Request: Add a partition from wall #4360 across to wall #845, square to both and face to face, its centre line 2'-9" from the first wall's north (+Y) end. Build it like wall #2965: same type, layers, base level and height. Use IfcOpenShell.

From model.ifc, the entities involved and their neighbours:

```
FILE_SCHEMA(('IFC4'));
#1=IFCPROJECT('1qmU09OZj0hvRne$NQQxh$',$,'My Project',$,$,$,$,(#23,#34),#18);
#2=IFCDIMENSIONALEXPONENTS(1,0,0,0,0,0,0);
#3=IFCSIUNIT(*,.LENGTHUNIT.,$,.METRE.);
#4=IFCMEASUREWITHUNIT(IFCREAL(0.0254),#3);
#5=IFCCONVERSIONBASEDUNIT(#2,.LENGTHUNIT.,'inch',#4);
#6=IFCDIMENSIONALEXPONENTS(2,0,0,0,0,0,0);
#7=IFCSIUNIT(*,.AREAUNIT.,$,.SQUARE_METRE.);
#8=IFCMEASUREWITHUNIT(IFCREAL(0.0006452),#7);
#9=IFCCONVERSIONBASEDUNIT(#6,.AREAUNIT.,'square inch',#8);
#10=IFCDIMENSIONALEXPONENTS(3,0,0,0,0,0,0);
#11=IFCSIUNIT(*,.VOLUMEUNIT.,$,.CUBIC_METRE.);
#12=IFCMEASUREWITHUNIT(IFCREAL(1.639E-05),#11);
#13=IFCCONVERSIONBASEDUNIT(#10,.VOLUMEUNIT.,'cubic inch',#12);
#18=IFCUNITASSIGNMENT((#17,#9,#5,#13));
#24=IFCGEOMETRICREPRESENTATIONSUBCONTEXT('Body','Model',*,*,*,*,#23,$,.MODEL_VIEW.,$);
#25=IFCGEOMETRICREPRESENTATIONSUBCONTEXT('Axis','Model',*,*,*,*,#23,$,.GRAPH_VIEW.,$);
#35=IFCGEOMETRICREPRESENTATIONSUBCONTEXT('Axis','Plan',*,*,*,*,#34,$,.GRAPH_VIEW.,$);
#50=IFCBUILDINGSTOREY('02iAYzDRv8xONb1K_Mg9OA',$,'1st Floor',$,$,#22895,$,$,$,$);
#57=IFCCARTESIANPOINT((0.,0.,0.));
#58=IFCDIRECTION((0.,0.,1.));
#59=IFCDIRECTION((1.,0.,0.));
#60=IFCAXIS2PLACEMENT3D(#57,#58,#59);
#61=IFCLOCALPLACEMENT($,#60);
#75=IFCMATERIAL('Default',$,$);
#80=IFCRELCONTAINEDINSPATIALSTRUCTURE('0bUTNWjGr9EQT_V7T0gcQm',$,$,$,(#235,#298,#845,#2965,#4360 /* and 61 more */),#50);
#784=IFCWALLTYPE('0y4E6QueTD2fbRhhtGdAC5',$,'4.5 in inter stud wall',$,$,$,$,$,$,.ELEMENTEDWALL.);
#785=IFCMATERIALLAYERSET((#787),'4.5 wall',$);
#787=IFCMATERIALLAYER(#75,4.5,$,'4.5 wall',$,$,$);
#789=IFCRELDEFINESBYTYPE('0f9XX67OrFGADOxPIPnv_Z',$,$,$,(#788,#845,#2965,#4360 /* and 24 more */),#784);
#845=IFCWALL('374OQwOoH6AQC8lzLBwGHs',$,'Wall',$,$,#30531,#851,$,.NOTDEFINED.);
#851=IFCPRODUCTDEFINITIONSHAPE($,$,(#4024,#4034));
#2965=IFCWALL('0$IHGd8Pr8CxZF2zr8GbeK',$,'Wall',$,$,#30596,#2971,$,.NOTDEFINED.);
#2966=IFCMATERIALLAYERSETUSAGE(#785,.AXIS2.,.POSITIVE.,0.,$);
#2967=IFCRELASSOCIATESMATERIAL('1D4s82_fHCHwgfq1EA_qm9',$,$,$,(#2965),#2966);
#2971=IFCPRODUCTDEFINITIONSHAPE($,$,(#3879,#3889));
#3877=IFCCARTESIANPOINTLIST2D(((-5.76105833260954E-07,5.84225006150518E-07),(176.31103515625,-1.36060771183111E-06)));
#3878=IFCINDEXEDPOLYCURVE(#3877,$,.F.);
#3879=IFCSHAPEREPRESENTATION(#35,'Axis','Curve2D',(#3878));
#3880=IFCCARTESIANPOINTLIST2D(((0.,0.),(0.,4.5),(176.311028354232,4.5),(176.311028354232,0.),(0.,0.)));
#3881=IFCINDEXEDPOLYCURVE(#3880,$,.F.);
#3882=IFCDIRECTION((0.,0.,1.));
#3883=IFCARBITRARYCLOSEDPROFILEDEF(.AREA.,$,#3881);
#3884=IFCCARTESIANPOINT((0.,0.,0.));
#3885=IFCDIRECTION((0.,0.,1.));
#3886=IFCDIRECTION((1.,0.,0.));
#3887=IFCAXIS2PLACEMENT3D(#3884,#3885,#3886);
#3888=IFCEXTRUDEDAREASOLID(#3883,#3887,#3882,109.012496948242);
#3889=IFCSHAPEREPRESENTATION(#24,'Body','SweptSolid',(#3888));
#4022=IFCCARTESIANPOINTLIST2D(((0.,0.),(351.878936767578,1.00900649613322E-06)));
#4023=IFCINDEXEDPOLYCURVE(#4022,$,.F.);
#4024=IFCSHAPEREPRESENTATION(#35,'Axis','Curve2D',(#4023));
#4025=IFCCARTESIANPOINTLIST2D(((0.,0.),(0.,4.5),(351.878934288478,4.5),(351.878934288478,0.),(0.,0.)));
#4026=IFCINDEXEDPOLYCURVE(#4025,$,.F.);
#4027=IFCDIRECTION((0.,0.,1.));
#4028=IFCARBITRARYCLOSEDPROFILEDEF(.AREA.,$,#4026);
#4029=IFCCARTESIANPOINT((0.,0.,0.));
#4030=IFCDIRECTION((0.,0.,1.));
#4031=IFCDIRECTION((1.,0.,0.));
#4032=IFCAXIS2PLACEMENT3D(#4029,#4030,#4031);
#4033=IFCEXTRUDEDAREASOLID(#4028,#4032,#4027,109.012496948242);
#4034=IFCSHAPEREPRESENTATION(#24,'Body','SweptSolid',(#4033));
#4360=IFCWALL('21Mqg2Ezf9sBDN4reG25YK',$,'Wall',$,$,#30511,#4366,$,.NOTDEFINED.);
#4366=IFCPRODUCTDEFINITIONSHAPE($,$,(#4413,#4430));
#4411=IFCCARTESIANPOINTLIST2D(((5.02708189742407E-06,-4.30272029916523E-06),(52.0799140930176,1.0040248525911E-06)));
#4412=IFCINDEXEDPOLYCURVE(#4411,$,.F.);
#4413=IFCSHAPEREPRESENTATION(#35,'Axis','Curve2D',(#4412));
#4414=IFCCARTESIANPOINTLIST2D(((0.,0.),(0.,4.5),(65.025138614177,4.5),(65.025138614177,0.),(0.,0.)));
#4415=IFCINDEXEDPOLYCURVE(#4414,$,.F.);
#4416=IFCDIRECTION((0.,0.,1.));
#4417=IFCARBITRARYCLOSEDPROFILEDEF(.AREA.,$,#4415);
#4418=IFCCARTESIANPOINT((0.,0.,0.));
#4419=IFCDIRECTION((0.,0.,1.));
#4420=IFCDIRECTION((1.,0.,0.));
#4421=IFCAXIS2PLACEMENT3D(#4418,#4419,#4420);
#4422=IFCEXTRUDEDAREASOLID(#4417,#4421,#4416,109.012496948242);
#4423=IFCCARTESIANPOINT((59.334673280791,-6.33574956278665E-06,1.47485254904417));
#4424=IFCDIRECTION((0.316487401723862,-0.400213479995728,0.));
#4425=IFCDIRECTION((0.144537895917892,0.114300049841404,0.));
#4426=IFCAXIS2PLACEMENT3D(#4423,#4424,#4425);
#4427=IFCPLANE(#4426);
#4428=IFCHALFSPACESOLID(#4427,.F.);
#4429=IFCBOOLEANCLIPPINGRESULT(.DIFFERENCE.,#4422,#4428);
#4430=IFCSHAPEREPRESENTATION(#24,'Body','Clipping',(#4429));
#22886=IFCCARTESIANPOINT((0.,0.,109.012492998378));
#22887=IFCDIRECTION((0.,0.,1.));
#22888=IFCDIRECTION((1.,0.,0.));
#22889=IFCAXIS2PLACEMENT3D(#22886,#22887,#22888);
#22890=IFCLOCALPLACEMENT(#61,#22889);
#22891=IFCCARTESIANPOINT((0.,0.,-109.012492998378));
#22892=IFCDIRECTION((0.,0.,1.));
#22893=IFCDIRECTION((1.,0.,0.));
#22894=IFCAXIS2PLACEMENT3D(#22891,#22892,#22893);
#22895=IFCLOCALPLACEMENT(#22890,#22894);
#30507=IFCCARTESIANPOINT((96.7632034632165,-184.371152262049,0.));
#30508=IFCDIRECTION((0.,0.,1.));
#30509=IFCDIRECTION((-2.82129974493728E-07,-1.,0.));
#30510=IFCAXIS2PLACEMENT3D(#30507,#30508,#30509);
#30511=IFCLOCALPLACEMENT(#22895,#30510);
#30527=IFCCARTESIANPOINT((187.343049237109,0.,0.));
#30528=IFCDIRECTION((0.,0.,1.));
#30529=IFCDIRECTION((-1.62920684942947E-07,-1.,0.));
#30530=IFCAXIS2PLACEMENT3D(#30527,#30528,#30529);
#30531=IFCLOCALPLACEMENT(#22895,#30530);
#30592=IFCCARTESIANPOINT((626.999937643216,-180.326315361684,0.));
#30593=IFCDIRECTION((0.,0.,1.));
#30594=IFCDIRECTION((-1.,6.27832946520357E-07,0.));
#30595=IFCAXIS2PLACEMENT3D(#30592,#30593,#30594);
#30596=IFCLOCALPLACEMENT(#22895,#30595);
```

```python
import numpy as np
import ifcopenshell
import ifcopenshell.api.geometry
import ifcopenshell.api.material
import ifcopenshell.api.pset
import ifcopenshell.api.root
import ifcopenshell.api.spatial
import ifcopenshell.api.type
import ifcopenshell.geom
import ifcopenshell.util.element
import ifcopenshell.util.placement
import ifcopenshell.util.representation
import ifcopenshell.util.shape
import ifcopenshell.util.unit

model = ifcopenshell.open("model.ifc")
unit_scale = ifcopenshell.util.unit.calculate_unit_scale(model)
settings = ifcopenshell.geom.settings()
settings.set("use-world-coords", True)

start_wall = model.by_guid("21Mqg2Ezf9sBDN4reG25YK")
end_wall = model.by_id(845)
like = model.by_guid("0$IHGd8Pr8CxZF2zr8GbeK")
matrix = ifcopenshell.util.placement.get_local_placement(start_wall.ObjectPlacement)
matrix[:3, 3] *= unit_scale


def extent(element):
    """Bounding box in the first wall's axes, in metres."""
    shape = ifcopenshell.geom.create_shape(settings, element)
    points = (ifcopenshell.util.shape.get_vertices(shape.geometry) - matrix[:3, 3]) @ matrix[:3, :3]
    return points.min(axis=0), points.max(axis=0)


y_start = extent(start_wall)[1][1]
y_end = extent(end_wall)[0][1]
like_min, like_max = extent(like)
length, height = float(abs(y_end - y_start)), float(like_max[2] - like_min[2])
layer_set = ifcopenshell.util.element.get_material(like, should_skip_usage=True)
thickness = sum(layer.LayerThickness for layer in layer_set.MaterialLayers) * unit_scale

wall = ifcopenshell.api.root.create_entity(model, ifc_class="IfcWall", name="New partition")
storey = ifcopenshell.util.element.get_container(like)
ifcopenshell.api.spatial.assign_container(model, products=[wall], relating_structure=storey)
ifcopenshell.api.type.assign_type(
    model, related_objects=[wall], relating_type=ifcopenshell.util.element.get_type(like), should_map_representations=False
)
rel = ifcopenshell.api.material.assign_material(
    model, products=[wall], type="IfcMaterialLayerSetUsage", material=layer_set
)
rel.RelatingMaterial.OffsetFromReferenceLine = -thickness / 2 / unit_scale
pset = ifcopenshell.api.pset.add_pset(model, product=wall, name="Pset_WallCommon")
ifcopenshell.api.pset.edit_pset(model, pset=pset, properties={"IsExternal": False, "LoadBearing": False})

# The axis runs down the middle of the wall.
axis = ifcopenshell.api.geometry.add_axis_representation(
    model, context=ifcopenshell.util.representation.get_context(model, "Model", "Axis"), axis=[(0.0, 0.0), (length, 0.0)]
)
body = ifcopenshell.api.geometry.add_wall_representation(
    model,
    context=ifcopenshell.util.representation.get_context(model, "Model", "Body", "MODEL_VIEW"),
    length=length,
    height=height,
    thickness=thickness,
    offset=-thickness / 2,
)
for representation in (axis, body):
    ifcopenshell.api.geometry.assign_representation(model, product=wall, representation=representation)

placement = matrix @ ifcopenshell.util.placement.rotation(90, "Z")
placement[:, 3] = matrix @ np.array([extent(start_wall)[0][0] + 0.8382, y_start, like_min[2], 1.0])
ifcopenshell.api.geometry.edit_object_placement(model, product=wall, matrix=placement)

print(f"partition {length:.3f} m long, {height:.3f} m high, {thickness:.3f} m thick")

model.write("model-out.ifc")
```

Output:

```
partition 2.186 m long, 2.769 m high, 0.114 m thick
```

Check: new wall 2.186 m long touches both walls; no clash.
